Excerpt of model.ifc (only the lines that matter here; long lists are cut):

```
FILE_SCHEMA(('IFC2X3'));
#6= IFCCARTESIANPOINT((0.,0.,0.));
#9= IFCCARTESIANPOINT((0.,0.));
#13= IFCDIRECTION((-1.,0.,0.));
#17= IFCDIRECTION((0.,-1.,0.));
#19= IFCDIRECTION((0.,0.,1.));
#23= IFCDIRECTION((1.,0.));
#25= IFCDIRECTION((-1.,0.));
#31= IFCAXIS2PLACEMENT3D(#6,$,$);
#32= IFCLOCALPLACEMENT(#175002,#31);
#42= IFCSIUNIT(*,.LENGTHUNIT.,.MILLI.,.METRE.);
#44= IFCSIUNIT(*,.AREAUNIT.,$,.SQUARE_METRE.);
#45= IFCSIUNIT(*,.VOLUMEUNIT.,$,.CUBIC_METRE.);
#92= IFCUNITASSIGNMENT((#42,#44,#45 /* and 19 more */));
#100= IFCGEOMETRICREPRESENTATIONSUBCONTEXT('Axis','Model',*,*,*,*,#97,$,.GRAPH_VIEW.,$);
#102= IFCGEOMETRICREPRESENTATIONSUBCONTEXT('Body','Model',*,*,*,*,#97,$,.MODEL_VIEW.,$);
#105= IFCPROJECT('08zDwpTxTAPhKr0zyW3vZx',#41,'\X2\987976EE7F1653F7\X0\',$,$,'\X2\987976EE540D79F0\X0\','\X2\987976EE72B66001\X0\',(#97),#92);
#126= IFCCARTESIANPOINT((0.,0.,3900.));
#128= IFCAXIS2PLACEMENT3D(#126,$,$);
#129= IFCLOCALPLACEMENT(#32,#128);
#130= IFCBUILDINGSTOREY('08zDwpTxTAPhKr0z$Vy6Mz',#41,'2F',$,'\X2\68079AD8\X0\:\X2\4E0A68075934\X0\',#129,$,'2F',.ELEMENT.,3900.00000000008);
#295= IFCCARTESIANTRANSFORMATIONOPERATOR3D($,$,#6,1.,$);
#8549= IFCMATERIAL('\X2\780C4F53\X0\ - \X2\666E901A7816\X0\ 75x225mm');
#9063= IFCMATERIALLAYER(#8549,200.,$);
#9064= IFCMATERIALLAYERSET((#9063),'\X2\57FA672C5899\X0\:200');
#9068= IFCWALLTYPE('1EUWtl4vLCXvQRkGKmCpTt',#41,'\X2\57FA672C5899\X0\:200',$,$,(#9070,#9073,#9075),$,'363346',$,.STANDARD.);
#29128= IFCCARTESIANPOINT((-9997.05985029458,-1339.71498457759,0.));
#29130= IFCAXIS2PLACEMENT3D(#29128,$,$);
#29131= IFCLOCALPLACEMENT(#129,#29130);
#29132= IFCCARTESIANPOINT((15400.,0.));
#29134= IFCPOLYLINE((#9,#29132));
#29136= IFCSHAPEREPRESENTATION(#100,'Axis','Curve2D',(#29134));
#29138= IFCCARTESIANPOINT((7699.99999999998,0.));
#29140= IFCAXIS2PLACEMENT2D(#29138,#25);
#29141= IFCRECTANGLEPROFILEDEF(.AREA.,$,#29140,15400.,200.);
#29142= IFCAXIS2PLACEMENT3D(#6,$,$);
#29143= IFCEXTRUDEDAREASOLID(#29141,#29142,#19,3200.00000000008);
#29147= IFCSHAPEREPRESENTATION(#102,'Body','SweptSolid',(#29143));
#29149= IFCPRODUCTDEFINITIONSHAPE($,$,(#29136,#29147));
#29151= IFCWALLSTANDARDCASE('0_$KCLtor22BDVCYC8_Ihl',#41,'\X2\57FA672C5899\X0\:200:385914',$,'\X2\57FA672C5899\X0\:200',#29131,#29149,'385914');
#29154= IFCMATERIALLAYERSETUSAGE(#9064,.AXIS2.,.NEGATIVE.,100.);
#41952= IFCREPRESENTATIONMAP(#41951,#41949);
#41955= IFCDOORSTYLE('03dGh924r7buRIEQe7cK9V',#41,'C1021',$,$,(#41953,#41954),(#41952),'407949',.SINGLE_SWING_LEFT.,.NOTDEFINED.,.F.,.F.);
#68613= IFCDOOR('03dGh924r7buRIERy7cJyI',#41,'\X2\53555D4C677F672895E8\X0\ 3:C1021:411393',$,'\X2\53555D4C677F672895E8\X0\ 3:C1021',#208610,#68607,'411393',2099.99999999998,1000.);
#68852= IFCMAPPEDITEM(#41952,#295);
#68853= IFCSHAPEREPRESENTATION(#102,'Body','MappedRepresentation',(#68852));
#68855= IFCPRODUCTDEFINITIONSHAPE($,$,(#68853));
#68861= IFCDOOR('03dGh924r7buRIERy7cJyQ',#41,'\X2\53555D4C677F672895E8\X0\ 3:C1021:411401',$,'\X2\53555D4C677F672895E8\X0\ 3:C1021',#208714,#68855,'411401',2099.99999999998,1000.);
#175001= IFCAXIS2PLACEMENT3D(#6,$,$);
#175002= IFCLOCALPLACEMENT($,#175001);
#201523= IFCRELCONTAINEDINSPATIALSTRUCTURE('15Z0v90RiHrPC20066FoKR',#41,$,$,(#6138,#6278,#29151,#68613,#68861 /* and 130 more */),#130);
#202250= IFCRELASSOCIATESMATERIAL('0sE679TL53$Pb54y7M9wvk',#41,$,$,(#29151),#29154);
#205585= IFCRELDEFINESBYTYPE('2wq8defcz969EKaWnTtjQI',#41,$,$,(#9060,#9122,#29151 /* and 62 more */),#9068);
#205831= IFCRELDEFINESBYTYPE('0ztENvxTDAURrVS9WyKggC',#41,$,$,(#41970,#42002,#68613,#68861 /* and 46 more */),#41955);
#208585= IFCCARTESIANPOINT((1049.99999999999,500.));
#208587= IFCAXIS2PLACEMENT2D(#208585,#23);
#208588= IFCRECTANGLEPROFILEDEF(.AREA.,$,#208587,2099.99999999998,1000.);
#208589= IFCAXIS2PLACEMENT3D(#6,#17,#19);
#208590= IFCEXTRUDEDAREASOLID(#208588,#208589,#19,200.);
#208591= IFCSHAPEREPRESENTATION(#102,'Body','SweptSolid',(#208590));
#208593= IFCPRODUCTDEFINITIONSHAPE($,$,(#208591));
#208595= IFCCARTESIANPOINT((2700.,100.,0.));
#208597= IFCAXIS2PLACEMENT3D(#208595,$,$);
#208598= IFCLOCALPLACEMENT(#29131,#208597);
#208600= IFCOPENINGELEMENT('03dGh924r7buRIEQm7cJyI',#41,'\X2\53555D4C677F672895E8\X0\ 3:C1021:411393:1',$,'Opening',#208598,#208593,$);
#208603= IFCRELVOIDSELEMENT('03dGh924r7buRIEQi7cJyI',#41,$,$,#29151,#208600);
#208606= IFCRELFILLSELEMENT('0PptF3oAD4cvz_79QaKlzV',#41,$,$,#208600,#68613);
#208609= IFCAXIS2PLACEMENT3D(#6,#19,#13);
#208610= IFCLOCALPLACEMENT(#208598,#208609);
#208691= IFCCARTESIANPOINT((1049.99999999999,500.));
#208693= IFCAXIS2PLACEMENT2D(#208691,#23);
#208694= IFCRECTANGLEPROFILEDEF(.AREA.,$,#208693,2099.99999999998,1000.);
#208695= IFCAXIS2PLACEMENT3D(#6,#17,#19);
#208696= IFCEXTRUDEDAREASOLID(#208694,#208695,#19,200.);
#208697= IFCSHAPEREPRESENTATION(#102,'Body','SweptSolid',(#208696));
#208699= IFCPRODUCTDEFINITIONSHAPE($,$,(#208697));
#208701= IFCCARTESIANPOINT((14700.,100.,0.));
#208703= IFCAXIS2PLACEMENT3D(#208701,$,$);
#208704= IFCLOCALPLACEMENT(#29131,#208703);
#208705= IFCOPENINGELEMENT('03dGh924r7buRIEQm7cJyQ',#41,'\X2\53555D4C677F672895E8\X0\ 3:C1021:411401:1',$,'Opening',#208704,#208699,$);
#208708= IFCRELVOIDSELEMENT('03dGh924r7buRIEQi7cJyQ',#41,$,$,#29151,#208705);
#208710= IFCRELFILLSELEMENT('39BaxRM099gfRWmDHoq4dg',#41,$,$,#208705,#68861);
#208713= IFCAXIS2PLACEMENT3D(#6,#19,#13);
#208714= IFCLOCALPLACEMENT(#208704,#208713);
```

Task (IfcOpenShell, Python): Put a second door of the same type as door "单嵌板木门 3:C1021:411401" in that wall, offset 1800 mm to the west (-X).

```python
import ifcopenshell
import ifcopenshell.api.feature
import ifcopenshell.api.geometry
import ifcopenshell.api.root
import ifcopenshell.geom
import ifcopenshell.util.element
import ifcopenshell.util.placement
import ifcopenshell.util.shape

model = ifcopenshell.open("model.ifc")
settings = ifcopenshell.geom.settings()


def volume(element):
    """Net volume in cubic metres, openings subtracted."""
    shape = ifcopenshell.geom.create_shape(settings, element)
    return ifcopenshell.util.shape.get_volume(shape.geometry)


def reuse_history(source, copy):
    """copy_class also copies each property set's owner history, people and application; keep the originals."""
    for rel in copy.IsDefinedBy:
        if rel.is_a("IfcRelDefinesByProperties") and (history := rel.RelatingPropertyDefinition.OwnerHistory):
            rel.RelatingPropertyDefinition.OwnerHistory = source.OwnerHistory
            ifcopenshell.util.element.remove_deep2(model, history)


door = model.by_id(68861)
opening = door.FillsVoids[0].RelatingOpeningElement
wall = opening.VoidsElements[0].RelatingBuildingElement
before = volume(wall)
shift = ifcopenshell.util.placement.get_local_placement(wall.ObjectPlacement)[:3, 0] * -1800.0

# copy_class copies the void relationship, type, container and properties, but no geometry.
new_opening = ifcopenshell.api.root.copy_class(model, product=opening)
new_opening.Representation = ifcopenshell.util.element.copy_deep(
    model, opening.Representation, exclude=["IfcGeometricRepresentationContext", "IfcRepresentationMap"]
)
new_opening.Name = "单嵌板木门 3:C1021"
new_door = ifcopenshell.api.root.copy_class(model, product=door)
new_door.Representation = ifcopenshell.util.element.copy_deep(
    model, door.Representation, exclude=["IfcGeometricRepresentationContext", "IfcRepresentationMap"]
)
new_door.Name = "单嵌板木门 3:C1021"
new_door.Tag = None
reuse_history(door, new_door)
fills = ifcopenshell.api.feature.add_filling(model, opening=new_opening, element=new_door)
fills.OwnerHistory = new_door.OwnerHistory  # required in IFC2X3

for old, new in ((opening, new_opening), (door, new_door)):
    matrix = ifcopenshell.util.placement.get_local_placement(old.ObjectPlacement)
    matrix[:3, 3] += shift
    ifcopenshell.api.geometry.edit_object_placement(model, product=new, matrix=matrix, is_si=False)

after = volume(wall)

print(f"wall volume {before:.3f} -> {after:.3f} m3")

model.write("model-out.ifc")
```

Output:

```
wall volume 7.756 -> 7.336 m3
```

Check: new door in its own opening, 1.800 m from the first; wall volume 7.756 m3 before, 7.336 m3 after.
